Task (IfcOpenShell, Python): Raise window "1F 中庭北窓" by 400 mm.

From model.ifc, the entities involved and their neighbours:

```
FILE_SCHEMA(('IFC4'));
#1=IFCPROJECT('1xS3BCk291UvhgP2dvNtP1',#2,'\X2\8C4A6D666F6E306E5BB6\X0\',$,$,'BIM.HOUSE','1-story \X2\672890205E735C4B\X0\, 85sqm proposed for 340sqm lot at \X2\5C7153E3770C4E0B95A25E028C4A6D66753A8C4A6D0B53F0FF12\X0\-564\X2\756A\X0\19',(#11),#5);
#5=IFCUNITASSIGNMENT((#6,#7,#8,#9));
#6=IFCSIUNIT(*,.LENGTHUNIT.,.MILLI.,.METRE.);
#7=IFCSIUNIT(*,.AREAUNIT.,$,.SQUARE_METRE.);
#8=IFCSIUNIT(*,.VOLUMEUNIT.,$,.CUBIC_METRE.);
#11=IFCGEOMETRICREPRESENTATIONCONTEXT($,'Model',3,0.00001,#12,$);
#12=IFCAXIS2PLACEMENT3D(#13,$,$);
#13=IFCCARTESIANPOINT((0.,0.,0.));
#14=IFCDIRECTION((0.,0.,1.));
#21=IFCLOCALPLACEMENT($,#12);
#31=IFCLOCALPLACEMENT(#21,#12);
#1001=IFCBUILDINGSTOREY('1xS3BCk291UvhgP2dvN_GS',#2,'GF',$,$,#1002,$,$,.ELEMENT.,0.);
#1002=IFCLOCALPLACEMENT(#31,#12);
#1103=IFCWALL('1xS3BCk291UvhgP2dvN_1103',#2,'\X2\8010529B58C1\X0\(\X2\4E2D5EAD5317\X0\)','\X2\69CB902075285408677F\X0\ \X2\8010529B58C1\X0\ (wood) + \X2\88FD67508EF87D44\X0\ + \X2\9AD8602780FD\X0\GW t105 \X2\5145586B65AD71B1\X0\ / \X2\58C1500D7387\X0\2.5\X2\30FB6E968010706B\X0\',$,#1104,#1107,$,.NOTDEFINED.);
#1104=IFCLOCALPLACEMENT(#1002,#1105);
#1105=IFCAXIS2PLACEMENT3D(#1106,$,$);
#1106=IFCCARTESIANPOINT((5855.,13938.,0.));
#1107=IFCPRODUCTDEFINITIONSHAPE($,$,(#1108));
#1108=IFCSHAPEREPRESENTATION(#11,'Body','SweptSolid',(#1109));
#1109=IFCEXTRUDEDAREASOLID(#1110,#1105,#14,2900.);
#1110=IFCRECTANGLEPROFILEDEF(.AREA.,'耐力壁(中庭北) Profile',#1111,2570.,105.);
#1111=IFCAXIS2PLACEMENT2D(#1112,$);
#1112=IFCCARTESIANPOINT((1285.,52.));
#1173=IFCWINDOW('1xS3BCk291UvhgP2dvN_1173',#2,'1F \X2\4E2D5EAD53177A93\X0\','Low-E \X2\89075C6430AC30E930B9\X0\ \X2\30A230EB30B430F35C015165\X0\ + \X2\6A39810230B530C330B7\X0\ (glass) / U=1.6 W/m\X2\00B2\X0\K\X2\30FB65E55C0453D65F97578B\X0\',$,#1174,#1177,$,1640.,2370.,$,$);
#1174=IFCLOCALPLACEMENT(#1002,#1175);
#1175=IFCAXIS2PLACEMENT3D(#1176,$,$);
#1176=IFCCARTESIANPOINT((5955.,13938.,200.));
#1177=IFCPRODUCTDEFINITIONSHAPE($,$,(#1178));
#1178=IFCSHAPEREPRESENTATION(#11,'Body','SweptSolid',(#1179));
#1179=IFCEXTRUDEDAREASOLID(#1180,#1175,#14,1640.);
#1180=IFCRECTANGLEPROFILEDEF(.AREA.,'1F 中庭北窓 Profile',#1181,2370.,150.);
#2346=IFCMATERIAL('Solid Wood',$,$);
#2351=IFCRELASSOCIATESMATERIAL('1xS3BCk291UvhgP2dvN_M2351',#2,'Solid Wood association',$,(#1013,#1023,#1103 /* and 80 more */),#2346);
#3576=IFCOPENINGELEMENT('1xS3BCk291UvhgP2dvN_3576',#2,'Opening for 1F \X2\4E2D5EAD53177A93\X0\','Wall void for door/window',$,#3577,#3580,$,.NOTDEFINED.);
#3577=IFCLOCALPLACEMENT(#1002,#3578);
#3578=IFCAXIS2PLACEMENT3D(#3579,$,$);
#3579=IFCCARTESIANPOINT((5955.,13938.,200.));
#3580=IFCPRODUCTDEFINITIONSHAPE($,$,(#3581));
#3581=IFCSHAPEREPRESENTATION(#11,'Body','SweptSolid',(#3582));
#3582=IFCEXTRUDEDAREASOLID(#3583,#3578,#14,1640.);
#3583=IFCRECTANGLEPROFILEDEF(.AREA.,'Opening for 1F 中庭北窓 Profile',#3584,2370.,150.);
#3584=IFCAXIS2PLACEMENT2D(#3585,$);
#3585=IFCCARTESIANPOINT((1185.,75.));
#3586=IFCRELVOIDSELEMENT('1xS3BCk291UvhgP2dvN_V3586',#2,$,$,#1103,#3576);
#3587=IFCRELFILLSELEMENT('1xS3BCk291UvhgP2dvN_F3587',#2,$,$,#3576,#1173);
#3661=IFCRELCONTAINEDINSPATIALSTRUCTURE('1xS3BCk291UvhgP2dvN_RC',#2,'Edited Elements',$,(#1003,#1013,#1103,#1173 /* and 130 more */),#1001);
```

```python
import numpy as np
import ifcopenshell
import ifcopenshell.api.geometry
import ifcopenshell.util.placement
import ifcopenshell.util.unit

model = ifcopenshell.open("model.ifc")
unit_scale = ifcopenshell.util.unit.calculate_unit_scale(model)

window = model.by_guid("1xS3BCk291UvhgP2dvN_1173")
opening = window.FillsVoids[0].RelatingOpeningElement
dz = 400.0

shift = np.array([0.0, 0.0, dz])
# The window is not placed relative to its opening, so move both.
for product in (opening, window):
    matrix = ifcopenshell.util.placement.get_local_placement(product.ObjectPlacement)
    matrix[:3, 3] += shift
    ifcopenshell.api.geometry.edit_object_placement(model, product=product, matrix=matrix, is_si=False)

print(f"moved by {dz * unit_scale:+.3f} m")

model.write("model_edited.ifc")
```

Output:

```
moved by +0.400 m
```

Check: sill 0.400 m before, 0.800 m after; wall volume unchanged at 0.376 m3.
